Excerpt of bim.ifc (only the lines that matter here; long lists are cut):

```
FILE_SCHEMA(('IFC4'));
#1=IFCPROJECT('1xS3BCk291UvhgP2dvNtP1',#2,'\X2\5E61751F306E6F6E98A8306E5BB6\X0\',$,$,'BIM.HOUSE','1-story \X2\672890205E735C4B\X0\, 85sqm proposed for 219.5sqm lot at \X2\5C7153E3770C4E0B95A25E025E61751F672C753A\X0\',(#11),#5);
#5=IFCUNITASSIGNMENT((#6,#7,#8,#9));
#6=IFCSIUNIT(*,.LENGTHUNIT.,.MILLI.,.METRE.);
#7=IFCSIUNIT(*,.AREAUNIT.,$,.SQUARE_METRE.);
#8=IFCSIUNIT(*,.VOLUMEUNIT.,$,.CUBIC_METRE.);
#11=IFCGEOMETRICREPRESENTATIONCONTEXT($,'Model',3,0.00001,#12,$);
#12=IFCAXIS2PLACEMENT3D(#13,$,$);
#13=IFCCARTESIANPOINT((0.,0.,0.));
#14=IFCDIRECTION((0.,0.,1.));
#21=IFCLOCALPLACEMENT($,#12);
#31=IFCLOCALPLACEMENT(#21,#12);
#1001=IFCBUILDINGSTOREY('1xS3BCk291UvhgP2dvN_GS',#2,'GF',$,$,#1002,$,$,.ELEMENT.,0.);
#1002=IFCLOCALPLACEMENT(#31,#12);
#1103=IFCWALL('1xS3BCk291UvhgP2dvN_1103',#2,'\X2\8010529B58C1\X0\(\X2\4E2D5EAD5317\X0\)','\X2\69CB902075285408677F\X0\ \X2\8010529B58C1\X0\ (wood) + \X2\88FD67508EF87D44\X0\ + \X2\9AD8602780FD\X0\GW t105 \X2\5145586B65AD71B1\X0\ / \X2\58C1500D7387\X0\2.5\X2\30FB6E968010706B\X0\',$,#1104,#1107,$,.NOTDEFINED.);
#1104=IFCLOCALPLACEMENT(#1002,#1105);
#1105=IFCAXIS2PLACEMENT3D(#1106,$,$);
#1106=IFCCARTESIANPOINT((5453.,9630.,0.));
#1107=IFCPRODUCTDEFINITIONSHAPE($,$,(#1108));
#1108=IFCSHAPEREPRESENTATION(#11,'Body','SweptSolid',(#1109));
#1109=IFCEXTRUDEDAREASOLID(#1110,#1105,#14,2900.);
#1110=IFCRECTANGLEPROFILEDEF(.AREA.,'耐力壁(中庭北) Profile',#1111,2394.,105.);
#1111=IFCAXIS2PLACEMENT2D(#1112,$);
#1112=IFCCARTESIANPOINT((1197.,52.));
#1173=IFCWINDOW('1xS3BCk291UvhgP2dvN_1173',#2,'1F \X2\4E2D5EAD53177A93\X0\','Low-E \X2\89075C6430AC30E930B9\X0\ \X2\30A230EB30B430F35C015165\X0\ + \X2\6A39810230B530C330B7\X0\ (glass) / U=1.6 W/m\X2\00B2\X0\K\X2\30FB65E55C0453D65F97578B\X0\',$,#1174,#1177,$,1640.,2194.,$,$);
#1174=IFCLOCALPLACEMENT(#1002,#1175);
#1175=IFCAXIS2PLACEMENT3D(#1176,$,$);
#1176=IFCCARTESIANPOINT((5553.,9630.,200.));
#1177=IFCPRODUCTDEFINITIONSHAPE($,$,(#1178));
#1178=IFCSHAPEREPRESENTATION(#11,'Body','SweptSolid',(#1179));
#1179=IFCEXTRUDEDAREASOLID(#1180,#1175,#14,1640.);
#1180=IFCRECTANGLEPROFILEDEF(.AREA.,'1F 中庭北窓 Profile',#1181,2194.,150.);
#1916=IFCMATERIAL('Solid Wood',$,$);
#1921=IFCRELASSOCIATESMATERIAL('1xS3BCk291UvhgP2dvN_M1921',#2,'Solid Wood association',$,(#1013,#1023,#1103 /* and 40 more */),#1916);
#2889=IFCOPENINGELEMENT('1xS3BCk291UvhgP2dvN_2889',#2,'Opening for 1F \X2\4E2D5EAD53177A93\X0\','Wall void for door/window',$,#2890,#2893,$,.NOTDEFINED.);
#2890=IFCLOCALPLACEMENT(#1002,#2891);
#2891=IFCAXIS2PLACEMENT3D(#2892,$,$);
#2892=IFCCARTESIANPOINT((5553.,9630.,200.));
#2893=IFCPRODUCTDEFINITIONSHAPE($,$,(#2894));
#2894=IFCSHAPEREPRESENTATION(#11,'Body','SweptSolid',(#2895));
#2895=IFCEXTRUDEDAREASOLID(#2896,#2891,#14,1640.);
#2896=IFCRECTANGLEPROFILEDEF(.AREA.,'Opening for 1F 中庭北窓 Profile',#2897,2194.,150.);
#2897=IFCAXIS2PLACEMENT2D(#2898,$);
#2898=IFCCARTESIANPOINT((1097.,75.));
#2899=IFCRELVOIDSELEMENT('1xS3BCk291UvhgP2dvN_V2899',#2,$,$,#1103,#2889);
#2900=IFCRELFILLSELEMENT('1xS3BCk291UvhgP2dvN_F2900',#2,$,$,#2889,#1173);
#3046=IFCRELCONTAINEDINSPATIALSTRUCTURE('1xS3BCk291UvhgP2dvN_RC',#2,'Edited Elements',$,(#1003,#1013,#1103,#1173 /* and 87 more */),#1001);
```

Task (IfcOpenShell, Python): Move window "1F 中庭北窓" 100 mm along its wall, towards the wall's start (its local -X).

```python
import ifcopenshell
import ifcopenshell.api.geometry
import ifcopenshell.util.placement

model = ifcopenshell.open("bim.ifc")

window = model.by_id(1173)
opening = window.FillsVoids[0].RelatingOpeningElement
wall = opening.VoidsElements[0].RelatingBuildingElement

wall_matrix = ifcopenshell.util.placement.get_local_placement(wall.ObjectPlacement)
shift = wall_matrix[:3, 0] * -100.0
before = ifcopenshell.util.placement.get_local_placement(window.ObjectPlacement)[:3, 3].copy()

# The window is not placed relative to its opening, so move both.
for product in (opening, window):
    matrix = ifcopenshell.util.placement.get_local_placement(product.ObjectPlacement)
    matrix[:3, 3] += shift
    ifcopenshell.api.geometry.edit_object_placement(model, product=product, matrix=matrix, is_si=False)

after = ifcopenshell.util.placement.get_local_placement(window.ObjectPlacement)[:3, 3]
print("window moved by", (after - before).round(3) + 0.0)

model.write("bim_v2.ifc")
```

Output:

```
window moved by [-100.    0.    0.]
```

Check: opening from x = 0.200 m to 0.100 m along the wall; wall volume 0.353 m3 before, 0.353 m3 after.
